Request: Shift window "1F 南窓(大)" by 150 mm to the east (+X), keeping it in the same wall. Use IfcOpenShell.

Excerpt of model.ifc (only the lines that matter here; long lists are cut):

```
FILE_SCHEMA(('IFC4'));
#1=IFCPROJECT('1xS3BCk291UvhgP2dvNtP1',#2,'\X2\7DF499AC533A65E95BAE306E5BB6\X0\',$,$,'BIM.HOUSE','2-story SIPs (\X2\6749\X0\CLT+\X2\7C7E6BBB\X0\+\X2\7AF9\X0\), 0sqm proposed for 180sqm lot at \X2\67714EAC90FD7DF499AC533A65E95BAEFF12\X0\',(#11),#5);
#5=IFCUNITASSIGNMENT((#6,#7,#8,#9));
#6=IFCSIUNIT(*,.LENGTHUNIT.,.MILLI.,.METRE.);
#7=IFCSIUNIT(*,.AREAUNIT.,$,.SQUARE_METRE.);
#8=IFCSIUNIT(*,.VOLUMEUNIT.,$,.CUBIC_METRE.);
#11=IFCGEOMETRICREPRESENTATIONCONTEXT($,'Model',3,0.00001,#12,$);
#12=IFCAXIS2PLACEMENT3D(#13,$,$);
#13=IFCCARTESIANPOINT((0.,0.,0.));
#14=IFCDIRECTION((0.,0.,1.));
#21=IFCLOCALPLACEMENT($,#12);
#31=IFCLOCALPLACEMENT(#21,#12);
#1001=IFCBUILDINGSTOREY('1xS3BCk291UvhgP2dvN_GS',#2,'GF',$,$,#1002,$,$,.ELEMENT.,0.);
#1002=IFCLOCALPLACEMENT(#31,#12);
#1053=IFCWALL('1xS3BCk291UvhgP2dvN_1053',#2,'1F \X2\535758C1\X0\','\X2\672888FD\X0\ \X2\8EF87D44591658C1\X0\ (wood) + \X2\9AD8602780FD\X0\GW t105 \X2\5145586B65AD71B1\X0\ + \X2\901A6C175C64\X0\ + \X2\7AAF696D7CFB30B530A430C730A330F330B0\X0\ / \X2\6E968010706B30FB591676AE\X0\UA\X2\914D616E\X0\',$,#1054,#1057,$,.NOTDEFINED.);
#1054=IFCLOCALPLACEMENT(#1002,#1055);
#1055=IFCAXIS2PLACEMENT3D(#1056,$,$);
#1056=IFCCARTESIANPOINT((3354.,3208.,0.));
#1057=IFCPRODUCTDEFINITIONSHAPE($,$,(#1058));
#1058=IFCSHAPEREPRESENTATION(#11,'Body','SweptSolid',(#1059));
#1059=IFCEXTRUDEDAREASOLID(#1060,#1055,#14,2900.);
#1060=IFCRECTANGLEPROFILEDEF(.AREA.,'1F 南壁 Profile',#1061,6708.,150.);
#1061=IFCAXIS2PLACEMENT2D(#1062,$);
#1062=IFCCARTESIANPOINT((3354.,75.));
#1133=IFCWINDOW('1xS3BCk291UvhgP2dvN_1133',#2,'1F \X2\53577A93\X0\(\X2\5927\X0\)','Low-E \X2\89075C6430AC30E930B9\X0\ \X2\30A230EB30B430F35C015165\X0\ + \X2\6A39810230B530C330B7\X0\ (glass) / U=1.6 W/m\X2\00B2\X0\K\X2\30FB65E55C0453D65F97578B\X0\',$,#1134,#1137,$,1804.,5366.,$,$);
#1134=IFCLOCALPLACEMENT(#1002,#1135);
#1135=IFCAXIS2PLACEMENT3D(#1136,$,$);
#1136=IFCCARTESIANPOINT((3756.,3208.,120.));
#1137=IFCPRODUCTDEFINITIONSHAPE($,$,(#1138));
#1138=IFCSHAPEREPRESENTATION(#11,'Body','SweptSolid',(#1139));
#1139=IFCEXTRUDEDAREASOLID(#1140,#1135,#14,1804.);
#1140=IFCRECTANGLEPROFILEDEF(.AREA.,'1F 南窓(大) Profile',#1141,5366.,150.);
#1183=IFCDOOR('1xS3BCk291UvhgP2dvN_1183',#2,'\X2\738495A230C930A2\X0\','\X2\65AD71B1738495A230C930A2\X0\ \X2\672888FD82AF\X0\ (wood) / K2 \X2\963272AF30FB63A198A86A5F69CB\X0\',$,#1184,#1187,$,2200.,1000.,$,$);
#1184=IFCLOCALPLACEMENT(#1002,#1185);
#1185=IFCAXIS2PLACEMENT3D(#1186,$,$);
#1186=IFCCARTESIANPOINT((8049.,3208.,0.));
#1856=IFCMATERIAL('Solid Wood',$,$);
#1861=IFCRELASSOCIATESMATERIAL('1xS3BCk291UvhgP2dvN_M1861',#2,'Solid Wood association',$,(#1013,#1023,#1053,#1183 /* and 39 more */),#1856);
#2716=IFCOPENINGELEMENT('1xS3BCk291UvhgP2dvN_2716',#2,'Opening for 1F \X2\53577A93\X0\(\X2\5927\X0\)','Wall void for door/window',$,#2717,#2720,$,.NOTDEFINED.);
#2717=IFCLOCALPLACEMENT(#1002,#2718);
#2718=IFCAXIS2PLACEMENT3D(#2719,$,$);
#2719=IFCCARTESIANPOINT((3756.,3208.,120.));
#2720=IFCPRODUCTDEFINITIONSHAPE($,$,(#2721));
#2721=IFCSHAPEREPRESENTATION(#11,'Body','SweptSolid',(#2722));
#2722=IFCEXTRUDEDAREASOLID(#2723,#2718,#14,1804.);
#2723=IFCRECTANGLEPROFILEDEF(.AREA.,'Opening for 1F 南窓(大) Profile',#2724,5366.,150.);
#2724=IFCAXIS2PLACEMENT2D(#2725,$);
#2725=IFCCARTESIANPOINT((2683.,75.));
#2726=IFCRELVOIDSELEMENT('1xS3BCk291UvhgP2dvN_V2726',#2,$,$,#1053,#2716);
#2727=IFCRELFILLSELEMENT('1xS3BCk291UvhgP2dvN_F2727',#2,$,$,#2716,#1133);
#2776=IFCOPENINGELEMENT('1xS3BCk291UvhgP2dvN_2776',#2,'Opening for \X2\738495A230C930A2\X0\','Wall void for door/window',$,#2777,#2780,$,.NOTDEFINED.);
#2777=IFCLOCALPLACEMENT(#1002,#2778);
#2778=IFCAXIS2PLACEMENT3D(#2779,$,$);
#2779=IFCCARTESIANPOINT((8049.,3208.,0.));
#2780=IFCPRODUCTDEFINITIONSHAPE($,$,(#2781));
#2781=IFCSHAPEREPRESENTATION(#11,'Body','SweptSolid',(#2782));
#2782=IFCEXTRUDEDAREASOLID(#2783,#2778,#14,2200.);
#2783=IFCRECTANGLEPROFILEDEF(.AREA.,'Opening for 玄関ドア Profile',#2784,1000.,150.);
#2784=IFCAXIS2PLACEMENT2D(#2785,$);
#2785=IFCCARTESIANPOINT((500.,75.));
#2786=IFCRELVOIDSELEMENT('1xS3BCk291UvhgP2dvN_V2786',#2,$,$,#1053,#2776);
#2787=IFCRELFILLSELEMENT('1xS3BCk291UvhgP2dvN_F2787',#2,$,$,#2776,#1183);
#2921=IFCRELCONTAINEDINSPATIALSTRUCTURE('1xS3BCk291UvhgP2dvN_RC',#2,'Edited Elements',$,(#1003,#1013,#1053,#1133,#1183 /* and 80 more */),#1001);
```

```python
import ifcopenshell
import ifcopenshell.api.geometry
import ifcopenshell.util.placement

model = ifcopenshell.open("model.ifc")

window = model.by_guid("1xS3BCk291UvhgP2dvN_1133")
opening = window.FillsVoids[0].RelatingOpeningElement
wall = opening.VoidsElements[0].RelatingBuildingElement

wall_matrix = ifcopenshell.util.placement.get_local_placement(wall.ObjectPlacement)
shift = wall_matrix[:3, 0] * 150.0
before = ifcopenshell.util.placement.get_local_placement(window.ObjectPlacement)[:3, 3].copy()

# The window is not placed relative to its opening, so move both.
for product in (opening, window):
    matrix = ifcopenshell.util.placement.get_local_placement(product.ObjectPlacement)
    matrix[:3, 3] += shift
    ifcopenshell.api.geometry.edit_object_placement(model, product=product, matrix=matrix, is_si=False)

after = ifcopenshell.util.placement.get_local_placement(window.ObjectPlacement)[:3, 3]
print("window moved by", (after - before).round(3) + 0.0)

model.write("model-out.ifc")
```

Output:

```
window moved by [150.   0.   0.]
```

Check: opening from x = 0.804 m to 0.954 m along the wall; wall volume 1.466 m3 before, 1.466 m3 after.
